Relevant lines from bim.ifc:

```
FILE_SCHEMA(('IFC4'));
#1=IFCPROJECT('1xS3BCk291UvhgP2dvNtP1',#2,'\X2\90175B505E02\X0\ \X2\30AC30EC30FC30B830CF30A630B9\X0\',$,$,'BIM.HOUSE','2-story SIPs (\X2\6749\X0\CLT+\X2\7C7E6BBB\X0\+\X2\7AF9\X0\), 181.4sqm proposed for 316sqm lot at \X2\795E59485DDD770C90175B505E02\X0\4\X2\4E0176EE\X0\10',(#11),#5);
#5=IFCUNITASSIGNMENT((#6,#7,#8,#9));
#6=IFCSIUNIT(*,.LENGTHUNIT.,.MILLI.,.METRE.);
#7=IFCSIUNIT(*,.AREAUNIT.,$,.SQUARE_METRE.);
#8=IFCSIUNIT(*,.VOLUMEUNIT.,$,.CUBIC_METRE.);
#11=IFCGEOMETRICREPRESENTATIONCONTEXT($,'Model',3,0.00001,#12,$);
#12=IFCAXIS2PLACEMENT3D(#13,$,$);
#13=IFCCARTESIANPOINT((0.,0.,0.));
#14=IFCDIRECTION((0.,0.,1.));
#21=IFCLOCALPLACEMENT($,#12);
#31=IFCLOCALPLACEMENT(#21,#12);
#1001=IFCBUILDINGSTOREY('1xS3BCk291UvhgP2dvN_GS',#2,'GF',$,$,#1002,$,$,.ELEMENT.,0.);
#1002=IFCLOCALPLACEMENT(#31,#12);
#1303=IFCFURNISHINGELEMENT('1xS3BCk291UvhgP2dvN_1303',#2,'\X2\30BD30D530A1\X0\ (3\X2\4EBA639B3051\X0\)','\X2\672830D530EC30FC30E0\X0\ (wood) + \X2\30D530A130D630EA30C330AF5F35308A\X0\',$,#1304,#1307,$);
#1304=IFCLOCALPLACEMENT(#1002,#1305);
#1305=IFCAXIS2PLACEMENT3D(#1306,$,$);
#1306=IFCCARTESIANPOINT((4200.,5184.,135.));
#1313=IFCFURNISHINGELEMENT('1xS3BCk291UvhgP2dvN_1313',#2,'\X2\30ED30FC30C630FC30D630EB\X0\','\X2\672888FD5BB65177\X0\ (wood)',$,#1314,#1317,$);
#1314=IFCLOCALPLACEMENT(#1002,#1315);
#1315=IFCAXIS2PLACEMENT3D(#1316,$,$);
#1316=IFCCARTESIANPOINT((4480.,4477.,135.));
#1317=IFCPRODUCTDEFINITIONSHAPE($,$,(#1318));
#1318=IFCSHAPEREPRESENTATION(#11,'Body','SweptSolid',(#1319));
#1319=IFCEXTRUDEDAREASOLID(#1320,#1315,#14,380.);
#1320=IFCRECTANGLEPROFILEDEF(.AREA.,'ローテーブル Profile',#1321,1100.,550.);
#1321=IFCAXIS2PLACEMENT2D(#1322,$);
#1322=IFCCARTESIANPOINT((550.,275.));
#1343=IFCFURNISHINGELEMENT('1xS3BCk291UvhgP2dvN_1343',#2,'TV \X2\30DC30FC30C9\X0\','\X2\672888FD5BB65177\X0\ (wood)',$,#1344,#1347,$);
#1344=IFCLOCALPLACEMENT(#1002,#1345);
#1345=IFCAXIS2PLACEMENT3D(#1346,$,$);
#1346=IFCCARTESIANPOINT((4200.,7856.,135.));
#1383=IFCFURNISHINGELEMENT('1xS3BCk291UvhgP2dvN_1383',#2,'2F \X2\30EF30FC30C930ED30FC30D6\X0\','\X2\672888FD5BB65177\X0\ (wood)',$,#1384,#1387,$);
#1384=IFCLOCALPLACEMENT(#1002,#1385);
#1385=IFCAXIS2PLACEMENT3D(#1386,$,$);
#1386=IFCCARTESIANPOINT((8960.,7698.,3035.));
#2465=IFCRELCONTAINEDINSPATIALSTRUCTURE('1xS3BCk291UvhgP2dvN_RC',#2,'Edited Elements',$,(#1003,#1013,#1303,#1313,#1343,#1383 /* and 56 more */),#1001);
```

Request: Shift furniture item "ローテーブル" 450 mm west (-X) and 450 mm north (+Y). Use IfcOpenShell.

```python
import ifcopenshell
import ifcopenshell.api.geometry
import ifcopenshell.util.placement

model = ifcopenshell.open("bim.ifc")

item = model.by_id(1313)
matrix = ifcopenshell.util.placement.get_local_placement(item.ObjectPlacement)
matrix[0, 3] -= 450.0
matrix[1, 3] += 450.0
ifcopenshell.api.geometry.edit_object_placement(model, product=item, matrix=matrix, is_si=False)

print(ifcopenshell.util.placement.get_local_placement(item.ObjectPlacement).round(3) + 0.0)

model.write("bim_v2.ifc")
```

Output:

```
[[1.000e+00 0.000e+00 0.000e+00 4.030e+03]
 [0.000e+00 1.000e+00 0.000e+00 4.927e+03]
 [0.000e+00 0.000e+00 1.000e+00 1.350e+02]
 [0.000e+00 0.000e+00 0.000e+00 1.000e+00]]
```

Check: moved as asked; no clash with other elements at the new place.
